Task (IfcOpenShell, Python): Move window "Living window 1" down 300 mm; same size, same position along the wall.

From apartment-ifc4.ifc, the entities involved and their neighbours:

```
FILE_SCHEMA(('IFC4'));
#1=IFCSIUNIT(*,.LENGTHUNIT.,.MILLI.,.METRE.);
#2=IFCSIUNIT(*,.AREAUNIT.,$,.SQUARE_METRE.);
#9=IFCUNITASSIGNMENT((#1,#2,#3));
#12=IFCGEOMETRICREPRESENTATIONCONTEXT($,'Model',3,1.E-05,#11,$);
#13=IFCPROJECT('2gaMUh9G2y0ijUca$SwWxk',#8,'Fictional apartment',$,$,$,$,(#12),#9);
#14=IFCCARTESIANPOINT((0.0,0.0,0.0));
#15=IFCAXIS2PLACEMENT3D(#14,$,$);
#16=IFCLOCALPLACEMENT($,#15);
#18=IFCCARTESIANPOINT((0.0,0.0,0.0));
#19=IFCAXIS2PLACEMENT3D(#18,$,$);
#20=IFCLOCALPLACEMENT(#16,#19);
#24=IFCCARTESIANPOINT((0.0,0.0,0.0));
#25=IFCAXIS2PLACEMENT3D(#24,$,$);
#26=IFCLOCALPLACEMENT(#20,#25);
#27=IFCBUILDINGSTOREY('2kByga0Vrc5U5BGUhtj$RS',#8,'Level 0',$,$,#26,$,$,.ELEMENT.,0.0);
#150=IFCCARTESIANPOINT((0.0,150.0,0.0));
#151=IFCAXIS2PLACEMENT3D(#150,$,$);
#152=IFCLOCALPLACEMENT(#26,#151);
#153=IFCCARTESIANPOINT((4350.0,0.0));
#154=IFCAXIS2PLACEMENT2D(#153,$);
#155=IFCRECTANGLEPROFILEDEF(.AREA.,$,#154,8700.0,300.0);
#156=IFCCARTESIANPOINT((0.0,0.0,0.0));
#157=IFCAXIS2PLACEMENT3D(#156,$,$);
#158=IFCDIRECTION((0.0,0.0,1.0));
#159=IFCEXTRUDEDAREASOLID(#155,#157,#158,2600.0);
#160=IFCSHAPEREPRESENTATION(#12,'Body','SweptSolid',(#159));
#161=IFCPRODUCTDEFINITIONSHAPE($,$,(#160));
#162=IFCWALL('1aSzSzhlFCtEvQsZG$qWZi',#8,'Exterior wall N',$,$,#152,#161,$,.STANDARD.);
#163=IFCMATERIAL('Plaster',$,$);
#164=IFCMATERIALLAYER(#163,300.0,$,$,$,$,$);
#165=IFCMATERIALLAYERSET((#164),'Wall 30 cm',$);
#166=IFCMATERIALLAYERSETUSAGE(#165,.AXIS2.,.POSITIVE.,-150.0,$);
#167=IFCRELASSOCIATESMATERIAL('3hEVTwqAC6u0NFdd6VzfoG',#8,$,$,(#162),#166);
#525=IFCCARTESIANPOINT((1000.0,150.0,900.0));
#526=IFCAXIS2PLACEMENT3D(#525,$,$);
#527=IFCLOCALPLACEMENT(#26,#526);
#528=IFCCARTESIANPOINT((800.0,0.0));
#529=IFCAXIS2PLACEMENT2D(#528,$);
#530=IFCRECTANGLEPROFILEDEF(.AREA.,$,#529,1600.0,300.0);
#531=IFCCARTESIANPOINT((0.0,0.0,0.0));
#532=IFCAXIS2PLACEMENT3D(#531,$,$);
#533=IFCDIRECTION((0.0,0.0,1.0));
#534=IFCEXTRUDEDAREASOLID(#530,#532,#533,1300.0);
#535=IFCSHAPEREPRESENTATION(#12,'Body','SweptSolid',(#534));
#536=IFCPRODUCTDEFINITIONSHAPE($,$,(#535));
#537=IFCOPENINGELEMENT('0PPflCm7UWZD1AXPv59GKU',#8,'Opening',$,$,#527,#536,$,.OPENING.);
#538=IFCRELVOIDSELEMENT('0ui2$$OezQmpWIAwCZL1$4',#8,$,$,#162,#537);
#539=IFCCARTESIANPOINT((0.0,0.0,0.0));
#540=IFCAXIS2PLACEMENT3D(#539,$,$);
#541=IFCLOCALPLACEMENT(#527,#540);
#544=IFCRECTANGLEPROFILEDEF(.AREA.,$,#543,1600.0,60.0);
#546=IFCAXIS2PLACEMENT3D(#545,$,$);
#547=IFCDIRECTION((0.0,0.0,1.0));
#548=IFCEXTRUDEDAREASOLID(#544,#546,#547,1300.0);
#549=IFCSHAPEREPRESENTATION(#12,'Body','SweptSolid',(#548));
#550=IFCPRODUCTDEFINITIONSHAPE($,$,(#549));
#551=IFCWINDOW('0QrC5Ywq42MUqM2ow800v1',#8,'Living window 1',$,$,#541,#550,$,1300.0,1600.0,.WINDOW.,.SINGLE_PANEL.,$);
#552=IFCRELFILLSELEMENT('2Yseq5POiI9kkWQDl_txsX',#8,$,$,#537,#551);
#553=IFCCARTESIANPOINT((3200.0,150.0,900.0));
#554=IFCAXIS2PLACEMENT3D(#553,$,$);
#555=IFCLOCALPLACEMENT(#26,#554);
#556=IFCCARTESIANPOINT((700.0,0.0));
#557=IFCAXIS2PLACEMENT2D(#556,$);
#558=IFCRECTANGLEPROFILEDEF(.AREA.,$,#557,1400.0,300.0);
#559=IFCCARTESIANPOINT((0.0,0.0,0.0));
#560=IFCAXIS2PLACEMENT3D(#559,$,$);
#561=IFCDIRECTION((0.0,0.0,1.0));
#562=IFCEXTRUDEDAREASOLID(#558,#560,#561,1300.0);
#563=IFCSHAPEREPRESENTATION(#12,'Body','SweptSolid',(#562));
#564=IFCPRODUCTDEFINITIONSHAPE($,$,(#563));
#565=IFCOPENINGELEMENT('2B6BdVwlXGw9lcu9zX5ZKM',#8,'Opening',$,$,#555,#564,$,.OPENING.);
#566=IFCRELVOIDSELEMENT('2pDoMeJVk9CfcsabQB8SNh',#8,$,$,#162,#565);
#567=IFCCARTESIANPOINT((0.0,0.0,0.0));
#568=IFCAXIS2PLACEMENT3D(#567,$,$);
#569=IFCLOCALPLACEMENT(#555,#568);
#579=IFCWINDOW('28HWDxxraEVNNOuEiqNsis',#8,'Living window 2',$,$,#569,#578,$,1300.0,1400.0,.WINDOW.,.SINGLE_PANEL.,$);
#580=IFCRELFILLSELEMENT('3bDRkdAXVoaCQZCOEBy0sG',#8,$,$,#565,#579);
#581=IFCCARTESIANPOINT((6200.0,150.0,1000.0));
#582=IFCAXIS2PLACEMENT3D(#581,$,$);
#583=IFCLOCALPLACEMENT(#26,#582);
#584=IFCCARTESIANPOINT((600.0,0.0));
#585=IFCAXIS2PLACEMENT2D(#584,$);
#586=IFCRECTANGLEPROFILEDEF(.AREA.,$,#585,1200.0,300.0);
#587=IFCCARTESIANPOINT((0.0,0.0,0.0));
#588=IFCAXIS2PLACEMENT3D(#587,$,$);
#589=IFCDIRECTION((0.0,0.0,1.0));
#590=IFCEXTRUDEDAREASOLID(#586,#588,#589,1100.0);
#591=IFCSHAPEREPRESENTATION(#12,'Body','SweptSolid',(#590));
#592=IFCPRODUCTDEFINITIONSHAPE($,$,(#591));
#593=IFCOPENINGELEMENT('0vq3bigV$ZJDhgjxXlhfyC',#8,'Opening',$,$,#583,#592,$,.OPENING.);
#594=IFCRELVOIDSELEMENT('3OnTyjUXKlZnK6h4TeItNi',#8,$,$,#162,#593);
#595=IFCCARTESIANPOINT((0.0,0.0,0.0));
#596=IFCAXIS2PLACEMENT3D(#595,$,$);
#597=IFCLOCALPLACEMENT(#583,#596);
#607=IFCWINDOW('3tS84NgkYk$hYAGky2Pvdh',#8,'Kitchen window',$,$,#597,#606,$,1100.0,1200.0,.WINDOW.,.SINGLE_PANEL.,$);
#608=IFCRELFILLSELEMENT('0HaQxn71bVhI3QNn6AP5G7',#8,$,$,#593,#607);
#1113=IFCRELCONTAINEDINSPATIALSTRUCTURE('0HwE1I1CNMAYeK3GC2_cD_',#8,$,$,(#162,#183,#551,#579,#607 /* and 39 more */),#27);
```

```python
import numpy as np
import ifcopenshell
import ifcopenshell.api.geometry
import ifcopenshell.util.placement
import ifcopenshell.util.unit

model = ifcopenshell.open("apartment-ifc4.ifc")
unit_scale = ifcopenshell.util.unit.calculate_unit_scale(model)

window = model.by_guid("0QrC5Ywq42MUqM2ow800v1")
opening = window.FillsVoids[0].RelatingOpeningElement
dz = -300.0

shift = np.array([0.0, 0.0, dz])
# The window is placed relative to its opening, so it follows when the opening moves.
matrix = ifcopenshell.util.placement.get_local_placement(opening.ObjectPlacement)
matrix[:3, 3] += shift
ifcopenshell.api.geometry.edit_object_placement(
    model, product=opening, matrix=matrix, is_si=False, should_transform_children=True
)

print(f"moved by {dz * unit_scale:+.3f} m")

model.write("apartment-ifc4_rev.ifc")
```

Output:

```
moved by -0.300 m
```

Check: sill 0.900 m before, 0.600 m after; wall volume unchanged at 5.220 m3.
